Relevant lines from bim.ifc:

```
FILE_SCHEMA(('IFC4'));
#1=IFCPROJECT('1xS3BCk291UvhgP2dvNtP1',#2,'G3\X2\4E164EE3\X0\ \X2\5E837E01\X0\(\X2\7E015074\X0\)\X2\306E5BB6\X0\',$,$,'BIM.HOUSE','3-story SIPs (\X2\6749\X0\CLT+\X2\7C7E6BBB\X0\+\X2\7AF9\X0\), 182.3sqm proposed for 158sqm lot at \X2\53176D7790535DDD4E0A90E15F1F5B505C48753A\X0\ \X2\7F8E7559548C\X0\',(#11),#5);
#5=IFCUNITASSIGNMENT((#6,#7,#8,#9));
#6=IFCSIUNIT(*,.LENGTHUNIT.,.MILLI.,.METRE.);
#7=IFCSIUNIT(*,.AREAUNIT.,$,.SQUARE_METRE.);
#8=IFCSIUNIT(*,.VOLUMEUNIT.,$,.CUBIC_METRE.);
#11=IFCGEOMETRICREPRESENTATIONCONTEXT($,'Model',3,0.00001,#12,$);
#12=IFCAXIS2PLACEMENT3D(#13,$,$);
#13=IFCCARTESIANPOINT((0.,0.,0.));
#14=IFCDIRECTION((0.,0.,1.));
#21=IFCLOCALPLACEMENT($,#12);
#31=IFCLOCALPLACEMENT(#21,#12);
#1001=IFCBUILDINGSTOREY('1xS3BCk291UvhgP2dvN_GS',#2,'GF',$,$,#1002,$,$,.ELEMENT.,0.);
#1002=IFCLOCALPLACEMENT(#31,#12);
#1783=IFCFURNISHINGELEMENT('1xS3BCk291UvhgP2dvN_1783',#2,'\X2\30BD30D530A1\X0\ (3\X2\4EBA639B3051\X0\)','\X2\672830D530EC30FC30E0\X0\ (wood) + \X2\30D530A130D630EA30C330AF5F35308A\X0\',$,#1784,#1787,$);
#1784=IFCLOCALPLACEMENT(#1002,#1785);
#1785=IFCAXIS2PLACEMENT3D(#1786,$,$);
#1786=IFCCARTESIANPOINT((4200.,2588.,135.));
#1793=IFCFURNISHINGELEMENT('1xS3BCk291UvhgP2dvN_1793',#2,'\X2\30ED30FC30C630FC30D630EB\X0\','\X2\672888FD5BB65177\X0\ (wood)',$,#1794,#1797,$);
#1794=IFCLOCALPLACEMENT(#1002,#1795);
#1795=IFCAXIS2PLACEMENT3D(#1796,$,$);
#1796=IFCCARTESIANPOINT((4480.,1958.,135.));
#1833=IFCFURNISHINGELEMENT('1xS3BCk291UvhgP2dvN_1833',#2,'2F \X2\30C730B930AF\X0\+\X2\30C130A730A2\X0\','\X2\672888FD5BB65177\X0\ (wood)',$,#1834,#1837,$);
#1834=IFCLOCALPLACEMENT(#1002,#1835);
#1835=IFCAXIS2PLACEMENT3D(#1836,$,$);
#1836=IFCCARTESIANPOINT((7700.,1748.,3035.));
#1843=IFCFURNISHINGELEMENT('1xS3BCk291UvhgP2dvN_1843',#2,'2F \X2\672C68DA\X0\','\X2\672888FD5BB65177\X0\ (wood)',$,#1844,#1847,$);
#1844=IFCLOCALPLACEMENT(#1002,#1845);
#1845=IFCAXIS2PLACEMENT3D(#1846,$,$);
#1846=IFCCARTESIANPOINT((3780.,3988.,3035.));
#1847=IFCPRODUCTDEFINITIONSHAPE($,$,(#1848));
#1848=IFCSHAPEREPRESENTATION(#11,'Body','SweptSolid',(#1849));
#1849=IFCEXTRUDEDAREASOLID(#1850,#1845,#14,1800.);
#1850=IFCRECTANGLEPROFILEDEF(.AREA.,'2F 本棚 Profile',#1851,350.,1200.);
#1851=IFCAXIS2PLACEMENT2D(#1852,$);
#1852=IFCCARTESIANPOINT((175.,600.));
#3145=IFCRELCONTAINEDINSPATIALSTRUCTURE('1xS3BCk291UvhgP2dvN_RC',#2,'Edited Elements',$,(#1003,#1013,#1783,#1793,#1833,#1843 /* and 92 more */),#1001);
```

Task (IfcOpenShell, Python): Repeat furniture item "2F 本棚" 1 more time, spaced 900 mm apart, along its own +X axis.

```python
import ifcopenshell
import ifcopenshell.api.geometry
import ifcopenshell.api.root
import ifcopenshell.util.element
import ifcopenshell.util.placement
import ifcopenshell.util.unit

model = ifcopenshell.open("bim.ifc")
unit_scale = ifcopenshell.util.unit.calculate_unit_scale(model)


def reuse_history(source, copy):
    """copy_class also copies each property set's owner history, people and application; keep the originals."""
    for rel in copy.IsDefinedBy:
        if rel.is_a("IfcRelDefinesByProperties") and (history := rel.RelatingPropertyDefinition.OwnerHistory):
            rel.RelatingPropertyDefinition.OwnerHistory = source.OwnerHistory
            ifcopenshell.util.element.remove_deep2(model, history)


source = model.by_id(1843)
base = ifcopenshell.util.placement.get_local_placement(source.ObjectPlacement)
step = base[:3, 0] * 0.9 / unit_scale

for i in range(1, 2):
    copy = ifcopenshell.api.root.copy_class(model, product=source)
    copy.Representation = ifcopenshell.util.element.copy_deep(
        model, source.Representation, exclude=["IfcGeometricRepresentationContext", "IfcRepresentationMap"]
    )
    reuse_history(source, copy)
    matrix = base.copy()
    matrix[:3, 3] += i * step
    print("added at", matrix[:3, 3].round(3) + 0.0)
    ifcopenshell.api.geometry.edit_object_placement(model, product=copy, matrix=matrix, is_si=False)

model.write("bim_v2.ifc")
```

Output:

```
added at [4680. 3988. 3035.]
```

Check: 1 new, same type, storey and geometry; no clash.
